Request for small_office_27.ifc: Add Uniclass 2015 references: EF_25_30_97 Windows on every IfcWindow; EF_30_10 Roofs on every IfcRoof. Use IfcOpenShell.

First a look at what the model holds.

```python
import ifcopenshell

model = ifcopenshell.open("small_office_27.ifc")
print(model.schema)
print("classifications:", [c.Name for c in model.by_type("IfcClassification")])
for ifc_class in ("IfcDoor", "IfcRoof", "IfcStair", "IfcWall", "IfcWindow"):
    print(ifc_class, len(model.by_type(ifc_class)))
```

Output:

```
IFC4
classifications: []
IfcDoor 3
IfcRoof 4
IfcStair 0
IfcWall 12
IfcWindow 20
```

```python
import ifcopenshell
import ifcopenshell.api.classification

model = ifcopenshell.open("small_office_27.ifc")

system = ifcopenshell.api.classification.add_classification(model, classification="Uniclass 2015")

codes = {
    "IfcWindow": ("EF_25_30_97", "Windows"),
    "IfcRoof": ("EF_30_10", "Roofs"),
}
for ifc_class, (code, name) in codes.items():
    products = model.by_type(ifc_class)
    ifcopenshell.api.classification.add_reference(
        model, products=products, classification=system, identification=code, name=name
    )
    print(code, len(products))

model.write("small_office_27_v2.ifc")
```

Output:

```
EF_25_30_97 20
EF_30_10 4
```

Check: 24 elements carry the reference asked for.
